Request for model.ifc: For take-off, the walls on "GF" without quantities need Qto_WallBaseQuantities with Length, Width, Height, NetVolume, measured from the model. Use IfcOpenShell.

First a look at what the model holds.

```python
import ifcopenshell
import ifcopenshell.util.element
import ifcopenshell.util.unit

model = ifcopenshell.open("model.ifc")
print(model.schema)
for unit_type in ("LENGTHUNIT", "AREAUNIT", "VOLUMEUNIT"):
    print(unit_type, ifcopenshell.util.unit.calculate_unit_scale(model, unit_type))
storey = next(s for s in model.by_type("IfcBuildingStorey") if s.Name == "GF")
walls = [e for e in ifcopenshell.util.element.get_decomposition(storey) if e.is_a("IfcWall")]
for e in sorted(walls, key=lambda e: e.id()):
    print(e.id(), e.is_a(), e.Name, list(ifcopenshell.util.element.get_psets(e, qtos_only=True)), sep=" | ")
```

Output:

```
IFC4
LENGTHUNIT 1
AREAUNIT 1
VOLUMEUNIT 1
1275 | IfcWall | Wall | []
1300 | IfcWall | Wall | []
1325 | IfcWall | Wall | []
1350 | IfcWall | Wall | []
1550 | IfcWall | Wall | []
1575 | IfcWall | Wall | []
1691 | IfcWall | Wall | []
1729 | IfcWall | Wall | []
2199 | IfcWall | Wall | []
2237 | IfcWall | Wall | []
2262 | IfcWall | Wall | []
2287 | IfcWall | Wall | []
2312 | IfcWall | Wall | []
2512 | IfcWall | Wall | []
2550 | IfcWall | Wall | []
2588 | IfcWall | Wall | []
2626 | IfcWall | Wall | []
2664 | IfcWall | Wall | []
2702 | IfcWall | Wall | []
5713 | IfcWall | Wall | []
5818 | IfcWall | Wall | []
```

```python
import ifcopenshell
import ifcopenshell.api.pset
import ifcopenshell.geom
import ifcopenshell.util.element
import ifcopenshell.util.shape
import ifcopenshell.util.unit

model = ifcopenshell.open("model.ifc")
unit_scale = ifcopenshell.util.unit.calculate_unit_scale(model)
volume_scale = ifcopenshell.util.unit.calculate_unit_scale(model, "VOLUMEUNIT")
settings = ifcopenshell.geom.settings()

storey = next(s for s in model.by_type("IfcBuildingStorey") if s.Name == "GF")
walls = [e for e in ifcopenshell.util.element.get_decomposition(storey) if e.is_a("IfcWall")]

for e in sorted(walls, key=lambda e: e.id()):
    if ifcopenshell.util.element.get_psets(e, qtos_only=True, should_inherit=False):
        continue
    # Geometry comes back in metres, in the element's own axes.
    shape = ifcopenshell.geom.create_shape(settings, e)
    values = {
        "Length": ifcopenshell.util.shape.get_x(shape.geometry) / unit_scale,
        "Width": ifcopenshell.util.shape.get_y(shape.geometry) / unit_scale,
        "Height": ifcopenshell.util.shape.get_z(shape.geometry) / unit_scale,
        "NetVolume": ifcopenshell.util.shape.get_volume(shape.geometry) / volume_scale,
    }
    qto = ifcopenshell.api.pset.add_qto(model, product=e, name="Qto_WallBaseQuantities")
    ifcopenshell.api.pset.edit_qto(model, qto=qto, properties=values)
    print(e.id(), {k: round(v, 3) for k, v in values.items()})

model.write("model-out.ifc")
```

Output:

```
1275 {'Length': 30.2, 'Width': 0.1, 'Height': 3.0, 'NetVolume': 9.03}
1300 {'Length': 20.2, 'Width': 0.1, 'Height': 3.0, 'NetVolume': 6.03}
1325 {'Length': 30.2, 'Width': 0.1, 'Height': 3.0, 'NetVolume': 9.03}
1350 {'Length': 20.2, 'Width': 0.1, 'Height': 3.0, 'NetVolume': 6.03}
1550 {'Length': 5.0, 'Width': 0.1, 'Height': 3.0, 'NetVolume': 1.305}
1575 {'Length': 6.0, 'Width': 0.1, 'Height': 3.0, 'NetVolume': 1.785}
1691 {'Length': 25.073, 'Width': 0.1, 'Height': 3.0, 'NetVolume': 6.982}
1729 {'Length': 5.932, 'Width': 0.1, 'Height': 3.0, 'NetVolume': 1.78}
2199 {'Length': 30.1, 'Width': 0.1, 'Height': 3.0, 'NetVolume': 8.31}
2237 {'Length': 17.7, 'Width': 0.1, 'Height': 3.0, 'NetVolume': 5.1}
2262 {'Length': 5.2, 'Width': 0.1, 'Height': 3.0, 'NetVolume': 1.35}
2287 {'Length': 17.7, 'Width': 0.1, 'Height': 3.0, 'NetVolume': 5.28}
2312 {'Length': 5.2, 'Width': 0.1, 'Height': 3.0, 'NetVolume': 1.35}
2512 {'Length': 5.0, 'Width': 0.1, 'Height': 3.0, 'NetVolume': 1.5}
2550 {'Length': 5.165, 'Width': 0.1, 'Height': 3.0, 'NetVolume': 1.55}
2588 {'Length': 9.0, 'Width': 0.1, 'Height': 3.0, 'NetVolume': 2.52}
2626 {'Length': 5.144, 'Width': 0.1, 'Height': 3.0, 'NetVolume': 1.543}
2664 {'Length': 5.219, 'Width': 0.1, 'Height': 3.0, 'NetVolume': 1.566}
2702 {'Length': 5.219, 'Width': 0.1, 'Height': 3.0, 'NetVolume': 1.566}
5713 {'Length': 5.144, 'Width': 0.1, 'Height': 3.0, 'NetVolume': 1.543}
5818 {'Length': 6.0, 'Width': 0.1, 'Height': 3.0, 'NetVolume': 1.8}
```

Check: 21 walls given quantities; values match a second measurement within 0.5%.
